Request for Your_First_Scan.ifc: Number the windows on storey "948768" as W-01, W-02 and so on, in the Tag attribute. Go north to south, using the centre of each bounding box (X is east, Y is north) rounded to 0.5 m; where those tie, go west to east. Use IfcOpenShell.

First a look at what the model holds.

```python
import ifcopenshell
import ifcopenshell.util.element
import ifcopenshell.util.placement

model = ifcopenshell.open("Your_First_Scan.ifc")
print(model.schema)
storey = next(s for s in model.by_type("IfcBuildingStorey") if s.Name == "948768")
windows = [e for e in ifcopenshell.util.element.get_decomposition(storey) if e.is_a("IfcWindow")]
for e in sorted(windows, key=lambda e: e.id()):
    origin = ifcopenshell.util.placement.get_local_placement(e.ObjectPlacement)[:3, 3]
    print(e.id(), e.Tag, e.Name, origin.round(2) + 0.0, sep=" | ")
```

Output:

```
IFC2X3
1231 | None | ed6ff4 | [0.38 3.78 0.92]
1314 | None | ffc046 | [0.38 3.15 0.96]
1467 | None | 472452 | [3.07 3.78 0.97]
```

```python
import ifcopenshell
import ifcopenshell.geom
import ifcopenshell.util.element
import ifcopenshell.util.shape

model = ifcopenshell.open("Your_First_Scan.ifc")
settings = ifcopenshell.geom.settings()
settings.set("use-world-coords", True)


def centre(element):
    shape = ifcopenshell.geom.create_shape(settings, element)
    return ifcopenshell.util.shape.get_bbox_centroid(shape.geometry)


storey = next(s for s in model.by_type("IfcBuildingStorey") if s.Name == "948768")
windows = [e for e in ifcopenshell.util.element.get_decomposition(storey) if e.is_a("IfcWindow")]

# Insertion points can sit at a corner or the storey origin, so sort by the geometry (in metres).
centres = {e: centre(e) for e in windows}
windows.sort(key=lambda e: (-round(centres[e][1] / 0.5), centres[e][0]))

for i, e in enumerate(windows, start=1):
    number = f"W-{i:02d}"
    e.Tag = number
    print(e.id(), number)

model.write("Your_First_Scan_rev.ifc")
```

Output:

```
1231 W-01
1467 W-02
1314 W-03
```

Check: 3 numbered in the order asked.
